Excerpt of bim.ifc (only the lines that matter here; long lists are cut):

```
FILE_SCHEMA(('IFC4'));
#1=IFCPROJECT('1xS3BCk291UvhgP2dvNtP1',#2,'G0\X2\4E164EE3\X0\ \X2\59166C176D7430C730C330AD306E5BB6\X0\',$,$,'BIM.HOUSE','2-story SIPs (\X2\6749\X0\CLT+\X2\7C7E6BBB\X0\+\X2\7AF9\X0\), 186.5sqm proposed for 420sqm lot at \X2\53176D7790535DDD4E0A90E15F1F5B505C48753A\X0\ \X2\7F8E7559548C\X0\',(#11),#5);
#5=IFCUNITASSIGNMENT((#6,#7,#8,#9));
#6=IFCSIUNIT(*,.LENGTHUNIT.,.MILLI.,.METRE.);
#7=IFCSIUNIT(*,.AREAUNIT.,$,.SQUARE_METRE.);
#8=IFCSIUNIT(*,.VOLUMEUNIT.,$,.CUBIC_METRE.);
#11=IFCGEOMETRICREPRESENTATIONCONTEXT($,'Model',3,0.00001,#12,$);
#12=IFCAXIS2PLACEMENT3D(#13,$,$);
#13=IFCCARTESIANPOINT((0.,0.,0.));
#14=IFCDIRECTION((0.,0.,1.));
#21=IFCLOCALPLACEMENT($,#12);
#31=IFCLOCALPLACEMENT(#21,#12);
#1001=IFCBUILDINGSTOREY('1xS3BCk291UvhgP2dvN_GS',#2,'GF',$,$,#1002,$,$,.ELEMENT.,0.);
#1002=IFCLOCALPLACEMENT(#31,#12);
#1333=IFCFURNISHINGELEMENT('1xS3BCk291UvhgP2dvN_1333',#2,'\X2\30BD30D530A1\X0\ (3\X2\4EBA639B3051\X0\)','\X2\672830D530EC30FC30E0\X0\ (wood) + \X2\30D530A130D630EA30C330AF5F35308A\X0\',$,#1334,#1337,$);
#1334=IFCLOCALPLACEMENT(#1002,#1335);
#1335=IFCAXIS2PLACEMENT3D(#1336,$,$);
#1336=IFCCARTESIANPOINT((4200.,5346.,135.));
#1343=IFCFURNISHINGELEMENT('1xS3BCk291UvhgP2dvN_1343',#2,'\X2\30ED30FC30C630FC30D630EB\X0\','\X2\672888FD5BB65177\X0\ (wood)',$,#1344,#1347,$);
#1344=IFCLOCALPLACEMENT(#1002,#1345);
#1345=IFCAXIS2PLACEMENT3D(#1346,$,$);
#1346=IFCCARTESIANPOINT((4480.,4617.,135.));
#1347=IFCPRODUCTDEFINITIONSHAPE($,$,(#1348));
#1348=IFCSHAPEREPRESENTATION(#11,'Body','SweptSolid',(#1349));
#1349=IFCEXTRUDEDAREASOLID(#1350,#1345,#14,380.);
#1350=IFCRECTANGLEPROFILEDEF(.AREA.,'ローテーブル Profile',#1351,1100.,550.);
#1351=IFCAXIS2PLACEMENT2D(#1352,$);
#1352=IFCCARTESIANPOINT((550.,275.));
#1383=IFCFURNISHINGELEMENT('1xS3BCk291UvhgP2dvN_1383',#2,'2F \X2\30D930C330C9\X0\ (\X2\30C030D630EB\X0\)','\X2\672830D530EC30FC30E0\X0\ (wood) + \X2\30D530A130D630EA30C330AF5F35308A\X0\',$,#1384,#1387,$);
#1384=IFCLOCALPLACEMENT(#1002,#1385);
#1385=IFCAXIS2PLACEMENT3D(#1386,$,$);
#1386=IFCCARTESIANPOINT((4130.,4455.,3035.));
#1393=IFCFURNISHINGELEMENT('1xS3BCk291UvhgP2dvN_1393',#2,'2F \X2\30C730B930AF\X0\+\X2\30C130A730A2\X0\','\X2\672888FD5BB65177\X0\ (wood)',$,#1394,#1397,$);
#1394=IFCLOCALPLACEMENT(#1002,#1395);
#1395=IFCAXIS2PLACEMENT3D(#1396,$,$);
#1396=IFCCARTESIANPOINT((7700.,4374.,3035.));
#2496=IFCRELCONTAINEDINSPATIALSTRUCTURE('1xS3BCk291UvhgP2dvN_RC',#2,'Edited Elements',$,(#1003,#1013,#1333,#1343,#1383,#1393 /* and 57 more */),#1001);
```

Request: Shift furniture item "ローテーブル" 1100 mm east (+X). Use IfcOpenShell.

```python
import ifcopenshell
import ifcopenshell.api.geometry
import ifcopenshell.util.placement
import ifcopenshell.util.unit

model = ifcopenshell.open("bim.ifc")
unit_scale = ifcopenshell.util.unit.calculate_unit_scale(model)

item = model.by_guid("1xS3BCk291UvhgP2dvN_1343")
matrix = ifcopenshell.util.placement.get_local_placement(item.ObjectPlacement)
matrix[0, 3] += 1.1 / unit_scale
ifcopenshell.api.geometry.edit_object_placement(model, product=item, matrix=matrix, is_si=False)

print(ifcopenshell.util.placement.get_local_placement(item.ObjectPlacement).round(3) + 0.0)

model.write("bim_v2.ifc")
```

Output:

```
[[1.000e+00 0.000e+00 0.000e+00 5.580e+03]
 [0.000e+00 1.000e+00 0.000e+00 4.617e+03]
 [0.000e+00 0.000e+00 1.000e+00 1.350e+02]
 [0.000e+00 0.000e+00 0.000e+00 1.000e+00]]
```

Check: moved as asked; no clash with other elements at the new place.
